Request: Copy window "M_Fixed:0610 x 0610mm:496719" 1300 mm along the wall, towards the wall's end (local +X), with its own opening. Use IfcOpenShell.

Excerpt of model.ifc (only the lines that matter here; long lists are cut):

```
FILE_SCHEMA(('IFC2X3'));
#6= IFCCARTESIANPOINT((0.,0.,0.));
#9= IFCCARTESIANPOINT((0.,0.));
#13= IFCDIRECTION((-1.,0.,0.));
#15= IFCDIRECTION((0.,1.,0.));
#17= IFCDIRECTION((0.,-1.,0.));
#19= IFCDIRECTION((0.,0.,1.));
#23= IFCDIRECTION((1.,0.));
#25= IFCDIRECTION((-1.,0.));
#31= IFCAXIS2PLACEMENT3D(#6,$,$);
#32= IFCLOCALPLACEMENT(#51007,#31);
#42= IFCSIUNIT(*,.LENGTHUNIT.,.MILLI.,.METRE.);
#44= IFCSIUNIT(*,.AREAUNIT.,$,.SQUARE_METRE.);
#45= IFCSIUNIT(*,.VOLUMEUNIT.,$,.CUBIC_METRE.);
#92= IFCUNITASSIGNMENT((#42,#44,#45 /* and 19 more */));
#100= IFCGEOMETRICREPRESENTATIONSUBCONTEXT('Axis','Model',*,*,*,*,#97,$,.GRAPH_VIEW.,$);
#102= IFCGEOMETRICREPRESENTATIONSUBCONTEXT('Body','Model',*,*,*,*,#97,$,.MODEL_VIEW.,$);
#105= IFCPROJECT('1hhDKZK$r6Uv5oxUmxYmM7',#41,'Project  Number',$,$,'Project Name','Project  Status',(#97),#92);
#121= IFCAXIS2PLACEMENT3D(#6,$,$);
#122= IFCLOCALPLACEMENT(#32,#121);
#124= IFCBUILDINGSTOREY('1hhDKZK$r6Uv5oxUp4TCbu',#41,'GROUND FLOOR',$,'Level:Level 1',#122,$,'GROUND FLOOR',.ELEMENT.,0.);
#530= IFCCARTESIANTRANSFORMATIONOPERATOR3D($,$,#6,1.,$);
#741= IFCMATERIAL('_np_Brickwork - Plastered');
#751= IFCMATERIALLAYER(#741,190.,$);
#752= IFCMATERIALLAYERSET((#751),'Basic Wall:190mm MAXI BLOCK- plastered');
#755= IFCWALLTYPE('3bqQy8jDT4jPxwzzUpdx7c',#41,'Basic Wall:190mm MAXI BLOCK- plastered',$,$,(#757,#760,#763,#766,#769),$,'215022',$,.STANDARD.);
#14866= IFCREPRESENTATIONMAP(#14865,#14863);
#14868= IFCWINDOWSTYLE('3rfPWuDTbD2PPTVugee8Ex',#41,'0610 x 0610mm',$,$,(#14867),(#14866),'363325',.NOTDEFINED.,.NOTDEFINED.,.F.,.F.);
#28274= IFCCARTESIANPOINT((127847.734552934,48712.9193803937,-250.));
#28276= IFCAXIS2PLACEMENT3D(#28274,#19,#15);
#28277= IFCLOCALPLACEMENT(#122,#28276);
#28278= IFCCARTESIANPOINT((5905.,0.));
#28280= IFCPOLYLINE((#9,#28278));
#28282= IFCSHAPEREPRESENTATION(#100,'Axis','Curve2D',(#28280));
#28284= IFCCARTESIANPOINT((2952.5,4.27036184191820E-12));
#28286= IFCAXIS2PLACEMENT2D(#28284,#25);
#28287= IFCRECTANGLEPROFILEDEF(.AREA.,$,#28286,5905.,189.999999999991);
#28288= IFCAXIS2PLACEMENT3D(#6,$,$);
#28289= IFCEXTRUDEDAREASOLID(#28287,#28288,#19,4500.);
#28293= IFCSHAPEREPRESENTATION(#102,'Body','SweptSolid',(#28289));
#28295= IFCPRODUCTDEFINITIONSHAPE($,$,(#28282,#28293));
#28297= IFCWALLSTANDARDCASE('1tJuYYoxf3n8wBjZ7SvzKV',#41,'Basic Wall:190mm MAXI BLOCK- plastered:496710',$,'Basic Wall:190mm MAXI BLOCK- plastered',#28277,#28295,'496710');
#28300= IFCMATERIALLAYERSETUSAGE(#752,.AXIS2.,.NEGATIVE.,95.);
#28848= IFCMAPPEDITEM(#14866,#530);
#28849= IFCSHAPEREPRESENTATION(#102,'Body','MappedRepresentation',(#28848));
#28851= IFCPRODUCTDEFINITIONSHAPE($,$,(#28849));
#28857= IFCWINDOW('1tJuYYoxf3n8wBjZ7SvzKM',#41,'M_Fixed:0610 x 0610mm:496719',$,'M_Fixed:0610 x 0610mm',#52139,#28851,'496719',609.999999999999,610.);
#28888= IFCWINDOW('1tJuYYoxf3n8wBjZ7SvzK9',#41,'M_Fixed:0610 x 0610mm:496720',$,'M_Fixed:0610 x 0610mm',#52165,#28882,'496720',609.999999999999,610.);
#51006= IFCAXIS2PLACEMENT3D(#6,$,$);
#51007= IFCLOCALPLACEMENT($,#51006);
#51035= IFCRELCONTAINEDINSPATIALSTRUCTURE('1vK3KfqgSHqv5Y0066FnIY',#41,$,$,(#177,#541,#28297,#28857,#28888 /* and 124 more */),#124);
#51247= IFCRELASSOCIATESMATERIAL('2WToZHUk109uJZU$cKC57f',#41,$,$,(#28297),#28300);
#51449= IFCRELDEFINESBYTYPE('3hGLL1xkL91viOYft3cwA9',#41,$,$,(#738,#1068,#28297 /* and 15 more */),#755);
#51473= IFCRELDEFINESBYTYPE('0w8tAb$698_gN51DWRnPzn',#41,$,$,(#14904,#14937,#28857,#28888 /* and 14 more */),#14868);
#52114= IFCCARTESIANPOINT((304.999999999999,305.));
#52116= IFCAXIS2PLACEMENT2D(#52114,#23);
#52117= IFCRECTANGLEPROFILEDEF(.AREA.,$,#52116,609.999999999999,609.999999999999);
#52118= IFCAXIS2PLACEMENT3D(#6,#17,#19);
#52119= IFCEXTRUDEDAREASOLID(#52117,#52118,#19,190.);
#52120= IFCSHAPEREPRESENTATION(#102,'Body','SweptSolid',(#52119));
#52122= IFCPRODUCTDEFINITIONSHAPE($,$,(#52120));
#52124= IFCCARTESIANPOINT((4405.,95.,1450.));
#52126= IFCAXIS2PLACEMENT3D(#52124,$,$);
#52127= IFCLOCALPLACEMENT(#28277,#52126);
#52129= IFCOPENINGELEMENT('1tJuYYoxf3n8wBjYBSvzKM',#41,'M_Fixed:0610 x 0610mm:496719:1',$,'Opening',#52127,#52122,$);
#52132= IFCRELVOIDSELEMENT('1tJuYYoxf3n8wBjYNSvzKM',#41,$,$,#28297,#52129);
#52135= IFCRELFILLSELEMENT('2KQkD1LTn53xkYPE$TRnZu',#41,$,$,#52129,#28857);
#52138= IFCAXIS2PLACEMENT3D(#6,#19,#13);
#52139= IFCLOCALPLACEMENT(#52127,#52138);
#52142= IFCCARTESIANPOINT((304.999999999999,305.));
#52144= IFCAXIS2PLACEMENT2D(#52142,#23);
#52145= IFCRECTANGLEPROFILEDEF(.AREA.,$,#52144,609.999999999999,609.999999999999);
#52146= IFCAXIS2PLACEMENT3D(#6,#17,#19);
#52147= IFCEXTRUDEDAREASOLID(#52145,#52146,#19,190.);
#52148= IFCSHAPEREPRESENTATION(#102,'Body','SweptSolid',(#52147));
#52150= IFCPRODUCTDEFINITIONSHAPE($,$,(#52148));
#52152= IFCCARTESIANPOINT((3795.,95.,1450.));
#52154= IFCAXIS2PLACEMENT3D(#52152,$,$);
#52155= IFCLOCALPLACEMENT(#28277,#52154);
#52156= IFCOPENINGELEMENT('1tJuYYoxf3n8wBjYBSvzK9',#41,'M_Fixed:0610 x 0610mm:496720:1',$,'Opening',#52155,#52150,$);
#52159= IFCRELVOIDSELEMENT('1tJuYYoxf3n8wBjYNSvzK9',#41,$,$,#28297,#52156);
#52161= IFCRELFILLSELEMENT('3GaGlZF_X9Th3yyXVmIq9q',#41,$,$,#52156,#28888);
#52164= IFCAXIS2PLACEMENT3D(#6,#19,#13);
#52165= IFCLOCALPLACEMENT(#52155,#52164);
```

```python
import ifcopenshell
import ifcopenshell.api.feature
import ifcopenshell.api.geometry
import ifcopenshell.api.root
import ifcopenshell.geom
import ifcopenshell.util.element
import ifcopenshell.util.placement
import ifcopenshell.util.shape

model = ifcopenshell.open("model.ifc")
settings = ifcopenshell.geom.settings()


def volume(element):
    """Net volume in cubic metres, openings subtracted."""
    shape = ifcopenshell.geom.create_shape(settings, element)
    return ifcopenshell.util.shape.get_volume(shape.geometry)


def reuse_history(source, copy):
    """copy_class also copies each property set's owner history, people and application; keep the originals."""
    for rel in copy.IsDefinedBy:
        if rel.is_a("IfcRelDefinesByProperties") and (history := rel.RelatingPropertyDefinition.OwnerHistory):
            rel.RelatingPropertyDefinition.OwnerHistory = source.OwnerHistory
            ifcopenshell.util.element.remove_deep2(model, history)


window = model.by_guid("1tJuYYoxf3n8wBjZ7SvzKM")
opening = window.FillsVoids[0].RelatingOpeningElement
wall = opening.VoidsElements[0].RelatingBuildingElement
before = volume(wall)
shift = ifcopenshell.util.placement.get_local_placement(wall.ObjectPlacement)[:3, 0] * 1300.0

# copy_class copies the void relationship, type, container and properties, but no geometry.
new_opening = ifcopenshell.api.root.copy_class(model, product=opening)
new_opening.Representation = ifcopenshell.util.element.copy_deep(
    model, opening.Representation, exclude=["IfcGeometricRepresentationContext", "IfcRepresentationMap"]
)
new_opening.Name = "M_Fixed:0610 x 0610mm"
new_window = ifcopenshell.api.root.copy_class(model, product=window)
new_window.Representation = ifcopenshell.util.element.copy_deep(
    model, window.Representation, exclude=["IfcGeometricRepresentationContext", "IfcRepresentationMap"]
)
new_window.Name = "M_Fixed:0610 x 0610mm"
new_window.Tag = None
reuse_history(window, new_window)
fills = ifcopenshell.api.feature.add_filling(model, opening=new_opening, element=new_window)
fills.OwnerHistory = new_window.OwnerHistory  # required in IFC2X3

for old, new in ((opening, new_opening), (window, new_window)):
    matrix = ifcopenshell.util.placement.get_local_placement(old.ObjectPlacement)
    matrix[:3, 3] += shift
    ifcopenshell.api.geometry.edit_object_placement(model, product=new, matrix=matrix, is_si=False)

after = volume(wall)

print(f"wall volume {before:.3f} -> {after:.3f} m3")

model.write("model_edited.ifc")
```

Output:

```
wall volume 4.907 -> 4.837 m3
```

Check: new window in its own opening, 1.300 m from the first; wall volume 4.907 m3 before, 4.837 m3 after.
